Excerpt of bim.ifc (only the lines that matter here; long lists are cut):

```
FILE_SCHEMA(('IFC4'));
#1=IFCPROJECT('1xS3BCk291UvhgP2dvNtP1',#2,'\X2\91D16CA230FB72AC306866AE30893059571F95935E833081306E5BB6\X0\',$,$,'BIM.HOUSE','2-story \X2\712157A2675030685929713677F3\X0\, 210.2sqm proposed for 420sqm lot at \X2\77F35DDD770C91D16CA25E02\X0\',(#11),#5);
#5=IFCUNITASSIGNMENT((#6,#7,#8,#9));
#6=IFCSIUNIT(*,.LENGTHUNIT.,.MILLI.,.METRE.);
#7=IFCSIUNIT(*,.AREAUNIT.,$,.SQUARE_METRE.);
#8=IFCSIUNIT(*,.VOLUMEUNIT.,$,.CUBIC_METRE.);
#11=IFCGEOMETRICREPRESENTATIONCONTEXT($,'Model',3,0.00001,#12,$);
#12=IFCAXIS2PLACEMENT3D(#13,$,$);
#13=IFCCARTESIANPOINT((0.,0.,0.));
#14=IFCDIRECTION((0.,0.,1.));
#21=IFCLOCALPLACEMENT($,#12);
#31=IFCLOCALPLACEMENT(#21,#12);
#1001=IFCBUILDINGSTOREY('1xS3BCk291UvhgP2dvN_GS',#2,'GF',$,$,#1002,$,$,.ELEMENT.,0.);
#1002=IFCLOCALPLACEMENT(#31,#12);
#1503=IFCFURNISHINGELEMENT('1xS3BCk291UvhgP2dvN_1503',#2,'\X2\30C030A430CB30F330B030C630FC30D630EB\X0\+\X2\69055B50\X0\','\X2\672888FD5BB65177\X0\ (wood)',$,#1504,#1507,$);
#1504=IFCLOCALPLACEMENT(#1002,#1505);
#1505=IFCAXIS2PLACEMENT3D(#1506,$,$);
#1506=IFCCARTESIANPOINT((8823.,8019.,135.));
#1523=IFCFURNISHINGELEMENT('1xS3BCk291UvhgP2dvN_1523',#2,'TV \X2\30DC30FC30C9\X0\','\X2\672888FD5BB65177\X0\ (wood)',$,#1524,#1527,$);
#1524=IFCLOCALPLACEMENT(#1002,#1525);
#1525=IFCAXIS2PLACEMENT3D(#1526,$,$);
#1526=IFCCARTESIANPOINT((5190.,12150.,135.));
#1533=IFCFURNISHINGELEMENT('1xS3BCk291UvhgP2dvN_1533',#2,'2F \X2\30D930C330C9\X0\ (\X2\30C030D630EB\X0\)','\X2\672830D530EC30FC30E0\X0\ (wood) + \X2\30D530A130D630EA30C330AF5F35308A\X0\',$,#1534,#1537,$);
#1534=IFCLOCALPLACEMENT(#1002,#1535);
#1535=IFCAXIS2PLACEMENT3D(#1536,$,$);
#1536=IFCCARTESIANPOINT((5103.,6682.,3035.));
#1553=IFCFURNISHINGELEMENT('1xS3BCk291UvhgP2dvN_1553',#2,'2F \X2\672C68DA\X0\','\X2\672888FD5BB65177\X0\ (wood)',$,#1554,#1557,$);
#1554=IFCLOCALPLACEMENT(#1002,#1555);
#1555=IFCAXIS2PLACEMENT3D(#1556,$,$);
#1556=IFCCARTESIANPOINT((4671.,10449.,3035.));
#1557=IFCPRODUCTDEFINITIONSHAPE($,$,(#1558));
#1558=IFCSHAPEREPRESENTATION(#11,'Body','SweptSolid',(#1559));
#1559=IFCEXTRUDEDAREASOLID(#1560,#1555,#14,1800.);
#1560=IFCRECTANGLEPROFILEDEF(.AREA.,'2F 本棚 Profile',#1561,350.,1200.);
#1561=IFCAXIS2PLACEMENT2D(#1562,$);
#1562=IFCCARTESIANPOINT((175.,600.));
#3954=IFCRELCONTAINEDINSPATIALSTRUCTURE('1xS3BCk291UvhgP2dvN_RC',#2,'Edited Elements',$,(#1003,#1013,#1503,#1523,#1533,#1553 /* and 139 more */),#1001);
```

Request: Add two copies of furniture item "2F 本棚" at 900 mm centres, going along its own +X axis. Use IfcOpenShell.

```python
import ifcopenshell
import ifcopenshell.api.geometry
import ifcopenshell.api.root
import ifcopenshell.util.element
import ifcopenshell.util.placement

model = ifcopenshell.open("bim.ifc")


def reuse_history(source, copy):
    """copy_class also copies each property set's owner history, people and application; keep the originals."""
    for rel in copy.IsDefinedBy:
        if rel.is_a("IfcRelDefinesByProperties") and (history := rel.RelatingPropertyDefinition.OwnerHistory):
            rel.RelatingPropertyDefinition.OwnerHistory = source.OwnerHistory
            ifcopenshell.util.element.remove_deep2(model, history)


source = model.by_guid("1xS3BCk291UvhgP2dvN_1553")
base = ifcopenshell.util.placement.get_local_placement(source.ObjectPlacement)
step = base[:3, 0] * 900.0

for i in range(1, 3):
    copy = ifcopenshell.api.root.copy_class(model, product=source)
    copy.Representation = ifcopenshell.util.element.copy_deep(
        model, source.Representation, exclude=["IfcGeometricRepresentationContext", "IfcRepresentationMap"]
    )
    reuse_history(source, copy)
    matrix = base.copy()
    matrix[:3, 3] += i * step
    print("added at", matrix[:3, 3].round(3) + 0.0)
    ifcopenshell.api.geometry.edit_object_placement(model, product=copy, matrix=matrix, is_si=False)

model.write("bim_edited.ifc")
```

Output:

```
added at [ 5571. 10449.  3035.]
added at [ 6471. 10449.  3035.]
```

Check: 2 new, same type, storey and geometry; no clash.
